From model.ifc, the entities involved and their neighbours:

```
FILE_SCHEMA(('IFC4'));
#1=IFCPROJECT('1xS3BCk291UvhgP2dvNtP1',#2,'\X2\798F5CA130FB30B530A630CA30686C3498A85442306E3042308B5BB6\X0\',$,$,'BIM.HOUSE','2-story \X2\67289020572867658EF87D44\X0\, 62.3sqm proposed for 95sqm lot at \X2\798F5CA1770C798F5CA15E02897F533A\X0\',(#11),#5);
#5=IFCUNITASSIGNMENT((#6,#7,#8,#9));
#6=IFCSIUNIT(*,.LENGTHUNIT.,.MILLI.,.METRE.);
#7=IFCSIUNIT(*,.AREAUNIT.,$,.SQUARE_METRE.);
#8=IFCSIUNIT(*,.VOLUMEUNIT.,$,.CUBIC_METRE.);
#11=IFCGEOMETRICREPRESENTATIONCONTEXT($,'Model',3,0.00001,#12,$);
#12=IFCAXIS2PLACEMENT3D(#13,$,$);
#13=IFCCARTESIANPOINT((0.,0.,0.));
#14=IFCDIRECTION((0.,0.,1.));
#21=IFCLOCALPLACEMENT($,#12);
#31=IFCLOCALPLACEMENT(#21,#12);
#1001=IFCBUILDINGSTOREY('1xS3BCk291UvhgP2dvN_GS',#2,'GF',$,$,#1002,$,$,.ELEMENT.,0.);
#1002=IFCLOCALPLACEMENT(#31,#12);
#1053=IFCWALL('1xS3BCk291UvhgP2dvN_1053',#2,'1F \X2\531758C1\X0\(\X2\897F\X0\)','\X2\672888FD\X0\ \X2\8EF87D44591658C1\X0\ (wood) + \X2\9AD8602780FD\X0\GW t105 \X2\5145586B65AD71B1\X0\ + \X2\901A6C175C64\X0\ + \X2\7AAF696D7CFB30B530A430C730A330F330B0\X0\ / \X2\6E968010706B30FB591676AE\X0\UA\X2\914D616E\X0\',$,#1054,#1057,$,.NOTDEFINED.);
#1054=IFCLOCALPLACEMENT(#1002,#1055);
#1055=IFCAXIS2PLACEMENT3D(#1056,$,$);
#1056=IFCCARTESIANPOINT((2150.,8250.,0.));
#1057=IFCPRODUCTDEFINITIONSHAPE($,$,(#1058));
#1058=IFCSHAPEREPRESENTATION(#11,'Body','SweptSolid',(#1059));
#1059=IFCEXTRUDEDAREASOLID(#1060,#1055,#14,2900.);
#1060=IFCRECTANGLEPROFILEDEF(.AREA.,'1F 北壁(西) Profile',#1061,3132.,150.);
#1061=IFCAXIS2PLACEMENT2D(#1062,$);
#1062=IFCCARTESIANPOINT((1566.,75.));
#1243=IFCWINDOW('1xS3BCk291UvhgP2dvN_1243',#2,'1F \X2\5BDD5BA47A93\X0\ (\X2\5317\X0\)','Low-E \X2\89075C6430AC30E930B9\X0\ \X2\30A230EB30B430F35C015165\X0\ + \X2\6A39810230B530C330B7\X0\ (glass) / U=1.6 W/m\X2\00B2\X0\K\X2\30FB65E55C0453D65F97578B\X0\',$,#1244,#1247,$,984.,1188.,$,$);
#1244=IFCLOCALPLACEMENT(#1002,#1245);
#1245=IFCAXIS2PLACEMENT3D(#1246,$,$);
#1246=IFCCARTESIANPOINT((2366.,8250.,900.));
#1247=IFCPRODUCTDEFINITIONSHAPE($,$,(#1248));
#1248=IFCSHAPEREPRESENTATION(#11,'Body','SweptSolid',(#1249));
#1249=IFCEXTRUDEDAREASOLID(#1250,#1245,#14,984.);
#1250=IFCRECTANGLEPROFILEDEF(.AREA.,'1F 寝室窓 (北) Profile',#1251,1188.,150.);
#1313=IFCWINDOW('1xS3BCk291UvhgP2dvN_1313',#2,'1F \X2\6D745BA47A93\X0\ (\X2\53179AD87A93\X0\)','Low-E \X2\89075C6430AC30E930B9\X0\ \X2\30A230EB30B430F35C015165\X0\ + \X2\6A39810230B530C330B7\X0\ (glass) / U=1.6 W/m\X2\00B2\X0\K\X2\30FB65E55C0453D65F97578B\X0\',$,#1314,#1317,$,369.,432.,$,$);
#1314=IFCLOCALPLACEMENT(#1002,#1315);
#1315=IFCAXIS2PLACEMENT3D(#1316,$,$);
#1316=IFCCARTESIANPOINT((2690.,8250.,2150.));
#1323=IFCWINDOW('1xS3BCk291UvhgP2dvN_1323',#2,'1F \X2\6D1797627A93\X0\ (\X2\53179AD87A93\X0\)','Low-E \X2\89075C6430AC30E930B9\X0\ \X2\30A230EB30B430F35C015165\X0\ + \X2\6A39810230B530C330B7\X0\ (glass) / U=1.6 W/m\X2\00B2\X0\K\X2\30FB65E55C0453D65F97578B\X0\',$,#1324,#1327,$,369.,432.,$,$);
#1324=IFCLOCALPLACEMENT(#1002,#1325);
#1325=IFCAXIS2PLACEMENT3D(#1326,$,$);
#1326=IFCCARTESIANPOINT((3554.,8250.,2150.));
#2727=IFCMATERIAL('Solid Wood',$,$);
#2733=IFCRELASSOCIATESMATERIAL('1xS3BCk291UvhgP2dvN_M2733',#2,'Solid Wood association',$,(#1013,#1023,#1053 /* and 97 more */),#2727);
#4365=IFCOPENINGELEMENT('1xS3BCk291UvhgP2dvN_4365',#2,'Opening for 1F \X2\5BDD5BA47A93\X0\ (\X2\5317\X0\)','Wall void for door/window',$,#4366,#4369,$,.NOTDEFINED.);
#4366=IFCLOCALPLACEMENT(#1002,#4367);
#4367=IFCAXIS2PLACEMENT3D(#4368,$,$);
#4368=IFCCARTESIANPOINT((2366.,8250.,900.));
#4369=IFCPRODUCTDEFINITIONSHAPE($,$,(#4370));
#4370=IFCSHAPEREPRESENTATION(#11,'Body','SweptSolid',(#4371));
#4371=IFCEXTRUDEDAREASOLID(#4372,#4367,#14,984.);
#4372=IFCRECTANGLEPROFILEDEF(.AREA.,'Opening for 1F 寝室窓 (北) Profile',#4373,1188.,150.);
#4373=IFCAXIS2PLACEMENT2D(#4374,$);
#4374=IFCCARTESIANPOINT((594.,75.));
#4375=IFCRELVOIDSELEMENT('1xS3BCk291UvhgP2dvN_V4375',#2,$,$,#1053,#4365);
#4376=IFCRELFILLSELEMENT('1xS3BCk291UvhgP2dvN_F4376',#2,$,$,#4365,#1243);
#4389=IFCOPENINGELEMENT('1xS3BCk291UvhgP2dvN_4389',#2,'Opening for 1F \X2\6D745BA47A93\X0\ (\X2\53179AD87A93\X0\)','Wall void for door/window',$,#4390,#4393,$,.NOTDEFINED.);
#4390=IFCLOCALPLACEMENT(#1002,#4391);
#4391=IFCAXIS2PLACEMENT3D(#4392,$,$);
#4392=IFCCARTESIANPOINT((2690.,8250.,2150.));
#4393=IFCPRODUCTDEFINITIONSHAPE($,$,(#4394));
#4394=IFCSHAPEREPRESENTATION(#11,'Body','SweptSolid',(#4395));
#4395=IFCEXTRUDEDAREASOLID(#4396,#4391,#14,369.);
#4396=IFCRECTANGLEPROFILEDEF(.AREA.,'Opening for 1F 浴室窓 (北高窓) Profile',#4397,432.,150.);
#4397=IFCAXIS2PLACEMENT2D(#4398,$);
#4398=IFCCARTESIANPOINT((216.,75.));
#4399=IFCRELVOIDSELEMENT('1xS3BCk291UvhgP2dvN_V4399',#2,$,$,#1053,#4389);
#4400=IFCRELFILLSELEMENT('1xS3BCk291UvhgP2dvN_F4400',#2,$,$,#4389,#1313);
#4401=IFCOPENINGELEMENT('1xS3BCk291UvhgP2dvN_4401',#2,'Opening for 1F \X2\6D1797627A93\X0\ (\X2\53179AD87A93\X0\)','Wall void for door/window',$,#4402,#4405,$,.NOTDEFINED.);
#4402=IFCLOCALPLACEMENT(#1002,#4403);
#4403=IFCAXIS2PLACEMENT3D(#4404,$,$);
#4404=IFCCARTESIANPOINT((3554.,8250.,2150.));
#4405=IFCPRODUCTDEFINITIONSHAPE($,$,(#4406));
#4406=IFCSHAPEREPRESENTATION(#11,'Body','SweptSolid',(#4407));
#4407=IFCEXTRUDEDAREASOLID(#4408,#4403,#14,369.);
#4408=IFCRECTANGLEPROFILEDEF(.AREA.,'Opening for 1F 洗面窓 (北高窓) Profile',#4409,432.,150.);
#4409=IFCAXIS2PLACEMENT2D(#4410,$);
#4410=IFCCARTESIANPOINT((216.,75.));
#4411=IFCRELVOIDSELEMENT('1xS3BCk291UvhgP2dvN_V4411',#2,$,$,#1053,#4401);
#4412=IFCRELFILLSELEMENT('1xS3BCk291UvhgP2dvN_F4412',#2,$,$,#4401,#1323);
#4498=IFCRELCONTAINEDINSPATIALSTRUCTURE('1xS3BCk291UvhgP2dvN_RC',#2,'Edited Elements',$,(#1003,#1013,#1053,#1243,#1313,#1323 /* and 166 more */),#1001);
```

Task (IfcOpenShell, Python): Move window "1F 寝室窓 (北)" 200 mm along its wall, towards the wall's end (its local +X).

```python
import ifcopenshell
import ifcopenshell.api.geometry
import ifcopenshell.util.placement
import ifcopenshell.util.unit

model = ifcopenshell.open("model.ifc")
unit_scale = ifcopenshell.util.unit.calculate_unit_scale(model)

window = model.by_guid("1xS3BCk291UvhgP2dvN_1243")
opening = window.FillsVoids[0].RelatingOpeningElement
wall = opening.VoidsElements[0].RelatingBuildingElement

wall_matrix = ifcopenshell.util.placement.get_local_placement(wall.ObjectPlacement)
shift = wall_matrix[:3, 0] * 0.2 / unit_scale
before = ifcopenshell.util.placement.get_local_placement(window.ObjectPlacement)[:3, 3].copy()

# The window is not placed relative to its opening, so move both.
for product in (opening, window):
    matrix = ifcopenshell.util.placement.get_local_placement(product.ObjectPlacement)
    matrix[:3, 3] += shift
    ifcopenshell.api.geometry.edit_object_placement(model, product=product, matrix=matrix, is_si=False)

after = ifcopenshell.util.placement.get_local_placement(window.ObjectPlacement)[:3, 3]
print("window moved by", (after - before).round(3) + 0.0)

model.write("model_edited.ifc")
```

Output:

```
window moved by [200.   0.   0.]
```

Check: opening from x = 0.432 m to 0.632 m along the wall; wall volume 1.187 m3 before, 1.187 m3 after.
